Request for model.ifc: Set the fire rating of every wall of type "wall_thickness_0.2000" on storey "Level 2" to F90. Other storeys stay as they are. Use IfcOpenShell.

First a look at what the model holds.

```python
import ifcopenshell
import ifcopenshell.util.element

model = ifcopenshell.open("model.ifc")
print(model.schema)
storey = next(s for s in model.by_type("IfcBuildingStorey") if s.Name == "Level 2")
walls = [e for e in ifcopenshell.util.element.get_decomposition(storey) if e.is_a("IfcWall")]
seen = {}
for e in walls:
    element_type = ifcopenshell.util.element.get_type(e)
    key = (element_type.Name if element_type != e and element_type else None, ifcopenshell.util.element.get_pset(e, "Pset_WallCommon", "FireRating"))
    seen[key] = seen.get(key, 0) + 1
for (name, value), count in sorted(seen.items(), key=str):
    print(count, "x", name, "|", value)
```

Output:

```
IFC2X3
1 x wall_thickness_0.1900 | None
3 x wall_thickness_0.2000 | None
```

```python
import ifcopenshell
import ifcopenshell.api.pset
import ifcopenshell.util.element

model = ifcopenshell.open("model.ifc")

storey = next(s for s in model.by_type("IfcBuildingStorey") if s.Name == "Level 2")
walls = [e for e in ifcopenshell.util.element.get_decomposition(storey) if e.is_a("IfcWall")]

count = 0
for e in walls:
    element_type = ifcopenshell.util.element.get_type(e)
    if element_type in (None, e) or element_type.Name != "wall_thickness_0.2000":
        continue
    # add_pset returns the element's existing set when there is one.
    pset = ifcopenshell.api.pset.add_pset(model, product=e, name="Pset_WallCommon")
    ifcopenshell.api.pset.edit_pset(model, pset=pset, properties={"FireRating": "F90"})
    count += 1

print(count, "walls updated")

model.write("model_v2.ifc")
```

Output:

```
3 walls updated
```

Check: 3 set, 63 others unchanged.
